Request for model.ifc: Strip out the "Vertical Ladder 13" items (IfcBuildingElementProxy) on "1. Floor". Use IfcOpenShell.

First a look at what the model holds.

```python
import ifcopenshell
import ifcopenshell.util.element

model = ifcopenshell.open("model.ifc")
print(model.schema)
storey = next(s for s in model.by_type("IfcBuildingStorey") if s.Name == "1. Floor")
proxies = [e for e in ifcopenshell.util.element.get_decomposition(storey) if e.is_a("IfcBuildingElementProxy")]
seen = {}
for e in proxies:
    element_type = ifcopenshell.util.element.get_type(e)
    name = element_type.Name if element_type not in (None, e) else None
    seen[name] = seen.get(name, 0) + 1
for name, count in sorted(seen.items(), key=str):
    print(count, "x", name)
```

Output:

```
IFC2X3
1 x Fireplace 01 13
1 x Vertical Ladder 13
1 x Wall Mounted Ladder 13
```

```python
import ifcopenshell
import ifcopenshell.api.root
import ifcopenshell.util.element

model = ifcopenshell.open("model.ifc")

storey = next(s for s in model.by_type("IfcBuildingStorey") if s.Name == "1. Floor")
proxies = [e for e in ifcopenshell.util.element.get_decomposition(storey) if e.is_a("IfcBuildingElementProxy")]
targets = [e for e in proxies if (t := ifcopenshell.util.element.get_type(e)) not in (None, e) and t.Name == "Vertical Ladder 13"]

for e in targets:
    ifcopenshell.api.root.remove_product(model, product=e)
print(len(targets), "removed")

model.write("model_rev.ifc")
```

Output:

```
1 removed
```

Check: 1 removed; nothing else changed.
